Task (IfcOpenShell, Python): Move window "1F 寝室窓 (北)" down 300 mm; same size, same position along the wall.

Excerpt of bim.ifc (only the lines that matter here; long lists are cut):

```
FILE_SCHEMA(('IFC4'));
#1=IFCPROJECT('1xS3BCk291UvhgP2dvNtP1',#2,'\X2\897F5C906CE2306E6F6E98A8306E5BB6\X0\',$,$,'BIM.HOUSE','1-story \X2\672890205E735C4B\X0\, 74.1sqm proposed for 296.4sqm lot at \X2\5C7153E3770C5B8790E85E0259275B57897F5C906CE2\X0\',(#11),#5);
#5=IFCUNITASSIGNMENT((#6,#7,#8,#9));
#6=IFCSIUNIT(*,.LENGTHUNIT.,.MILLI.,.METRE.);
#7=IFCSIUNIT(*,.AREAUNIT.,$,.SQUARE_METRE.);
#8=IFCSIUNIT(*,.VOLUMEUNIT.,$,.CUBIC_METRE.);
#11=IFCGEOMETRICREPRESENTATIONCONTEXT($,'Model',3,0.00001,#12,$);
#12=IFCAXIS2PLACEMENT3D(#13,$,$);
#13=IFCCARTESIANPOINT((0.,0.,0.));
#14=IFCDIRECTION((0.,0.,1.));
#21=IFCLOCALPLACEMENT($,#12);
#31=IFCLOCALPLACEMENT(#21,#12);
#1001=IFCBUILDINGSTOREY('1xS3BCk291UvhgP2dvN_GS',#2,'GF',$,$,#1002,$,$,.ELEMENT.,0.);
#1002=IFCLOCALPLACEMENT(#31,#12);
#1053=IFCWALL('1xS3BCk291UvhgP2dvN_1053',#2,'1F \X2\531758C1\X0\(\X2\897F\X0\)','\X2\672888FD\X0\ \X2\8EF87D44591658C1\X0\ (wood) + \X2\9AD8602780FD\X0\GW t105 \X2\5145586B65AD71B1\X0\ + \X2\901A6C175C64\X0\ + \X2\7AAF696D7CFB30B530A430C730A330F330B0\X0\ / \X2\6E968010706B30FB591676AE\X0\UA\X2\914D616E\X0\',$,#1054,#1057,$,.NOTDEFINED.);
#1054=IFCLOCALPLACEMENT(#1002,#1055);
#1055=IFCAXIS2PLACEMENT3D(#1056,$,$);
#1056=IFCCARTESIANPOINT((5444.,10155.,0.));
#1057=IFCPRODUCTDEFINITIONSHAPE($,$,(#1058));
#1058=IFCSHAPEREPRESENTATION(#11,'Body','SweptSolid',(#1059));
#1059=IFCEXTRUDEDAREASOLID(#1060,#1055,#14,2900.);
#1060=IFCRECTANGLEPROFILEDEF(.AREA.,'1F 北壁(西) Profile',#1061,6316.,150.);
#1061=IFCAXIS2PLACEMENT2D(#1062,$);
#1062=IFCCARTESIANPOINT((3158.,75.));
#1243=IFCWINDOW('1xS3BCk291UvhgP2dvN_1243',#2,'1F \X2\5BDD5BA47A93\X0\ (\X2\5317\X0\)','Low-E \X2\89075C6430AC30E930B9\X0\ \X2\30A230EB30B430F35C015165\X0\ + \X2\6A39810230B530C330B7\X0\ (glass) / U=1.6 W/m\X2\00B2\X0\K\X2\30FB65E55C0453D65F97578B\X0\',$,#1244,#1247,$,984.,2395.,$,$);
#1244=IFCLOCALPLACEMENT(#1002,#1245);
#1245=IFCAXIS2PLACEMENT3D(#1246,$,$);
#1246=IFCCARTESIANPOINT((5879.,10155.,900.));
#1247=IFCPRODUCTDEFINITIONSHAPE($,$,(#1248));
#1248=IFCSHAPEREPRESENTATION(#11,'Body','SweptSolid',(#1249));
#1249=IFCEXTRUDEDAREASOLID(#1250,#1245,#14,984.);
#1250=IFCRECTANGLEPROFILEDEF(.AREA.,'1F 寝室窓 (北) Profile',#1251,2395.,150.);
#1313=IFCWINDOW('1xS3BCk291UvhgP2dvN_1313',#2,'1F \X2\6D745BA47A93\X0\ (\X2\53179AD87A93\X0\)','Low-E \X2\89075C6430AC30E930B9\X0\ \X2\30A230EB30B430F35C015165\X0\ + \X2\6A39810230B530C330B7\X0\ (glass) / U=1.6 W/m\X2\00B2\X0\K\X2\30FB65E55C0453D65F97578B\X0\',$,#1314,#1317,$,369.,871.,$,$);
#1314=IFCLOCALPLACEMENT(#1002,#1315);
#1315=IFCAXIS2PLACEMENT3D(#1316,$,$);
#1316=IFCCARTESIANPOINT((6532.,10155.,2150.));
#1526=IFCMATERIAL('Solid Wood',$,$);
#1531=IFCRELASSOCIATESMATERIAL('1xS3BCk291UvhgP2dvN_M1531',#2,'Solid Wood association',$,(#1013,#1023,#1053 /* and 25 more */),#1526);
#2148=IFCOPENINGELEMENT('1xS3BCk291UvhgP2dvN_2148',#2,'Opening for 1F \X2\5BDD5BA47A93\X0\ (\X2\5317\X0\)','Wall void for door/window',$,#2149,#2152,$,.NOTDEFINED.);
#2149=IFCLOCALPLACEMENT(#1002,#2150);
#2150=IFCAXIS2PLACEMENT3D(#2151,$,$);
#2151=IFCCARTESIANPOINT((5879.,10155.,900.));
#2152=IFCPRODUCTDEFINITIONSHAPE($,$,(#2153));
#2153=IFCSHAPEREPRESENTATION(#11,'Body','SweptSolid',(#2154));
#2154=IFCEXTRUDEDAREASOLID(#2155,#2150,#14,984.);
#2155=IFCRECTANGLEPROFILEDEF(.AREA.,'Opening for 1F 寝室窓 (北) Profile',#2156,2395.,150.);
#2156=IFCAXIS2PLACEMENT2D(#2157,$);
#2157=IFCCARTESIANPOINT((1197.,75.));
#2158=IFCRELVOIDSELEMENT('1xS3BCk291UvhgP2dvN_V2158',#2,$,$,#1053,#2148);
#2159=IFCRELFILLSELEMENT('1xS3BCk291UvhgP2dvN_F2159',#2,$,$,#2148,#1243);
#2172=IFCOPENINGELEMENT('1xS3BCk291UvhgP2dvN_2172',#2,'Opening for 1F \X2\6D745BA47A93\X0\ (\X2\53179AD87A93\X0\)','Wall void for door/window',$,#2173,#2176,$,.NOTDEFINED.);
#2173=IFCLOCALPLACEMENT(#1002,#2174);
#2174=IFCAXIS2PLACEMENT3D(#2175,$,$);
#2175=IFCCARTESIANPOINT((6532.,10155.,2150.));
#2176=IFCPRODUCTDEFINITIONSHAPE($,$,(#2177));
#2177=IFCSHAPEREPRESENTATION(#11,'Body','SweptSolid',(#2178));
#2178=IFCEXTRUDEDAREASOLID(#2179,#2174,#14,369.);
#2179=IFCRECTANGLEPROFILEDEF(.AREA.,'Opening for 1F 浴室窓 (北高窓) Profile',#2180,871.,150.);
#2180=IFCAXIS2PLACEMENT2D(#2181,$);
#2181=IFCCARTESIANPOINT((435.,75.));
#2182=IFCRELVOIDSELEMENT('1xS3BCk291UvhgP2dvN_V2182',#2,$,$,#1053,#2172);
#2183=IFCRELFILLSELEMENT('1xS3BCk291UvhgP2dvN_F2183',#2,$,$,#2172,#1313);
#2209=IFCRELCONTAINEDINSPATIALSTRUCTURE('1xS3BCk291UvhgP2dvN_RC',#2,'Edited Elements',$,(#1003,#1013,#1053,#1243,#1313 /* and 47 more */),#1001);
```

```python
import numpy as np
import ifcopenshell
import ifcopenshell.api.geometry
import ifcopenshell.util.placement
import ifcopenshell.util.unit

model = ifcopenshell.open("bim.ifc")
unit_scale = ifcopenshell.util.unit.calculate_unit_scale(model)

window = model.by_guid("1xS3BCk291UvhgP2dvN_1243")
opening = window.FillsVoids[0].RelatingOpeningElement
dz = -300.0

shift = np.array([0.0, 0.0, dz])
# The window is not placed relative to its opening, so move both.
for product in (opening, window):
    matrix = ifcopenshell.util.placement.get_local_placement(product.ObjectPlacement)
    matrix[:3, 3] += shift
    ifcopenshell.api.geometry.edit_object_placement(model, product=product, matrix=matrix, is_si=False)

print(f"moved by {dz * unit_scale:+.3f} m")

model.write("bim-out.ifc")
```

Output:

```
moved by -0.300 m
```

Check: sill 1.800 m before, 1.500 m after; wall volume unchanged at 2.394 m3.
